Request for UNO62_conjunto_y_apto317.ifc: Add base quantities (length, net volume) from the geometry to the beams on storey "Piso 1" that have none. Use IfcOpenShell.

First a look at what the model holds.

```python
import ifcopenshell
import ifcopenshell.util.element
import ifcopenshell.util.unit

model = ifcopenshell.open("UNO62_conjunto_y_apto317.ifc")
print(model.schema)
for unit_type in ("LENGTHUNIT", "AREAUNIT", "VOLUMEUNIT"):
    print(unit_type, ifcopenshell.util.unit.calculate_unit_scale(model, unit_type))
storey = next(s for s in model.by_type("IfcBuildingStorey") if s.Name == "Piso 1")
beams = [e for e in ifcopenshell.util.element.get_decomposition(storey) if e.is_a("IfcBeam")]
for e in sorted(beams, key=lambda e: e.id()):
    print(e.id(), e.is_a(), e.Name, list(ifcopenshell.util.element.get_psets(e, qtos_only=True)), sep=" | ")
```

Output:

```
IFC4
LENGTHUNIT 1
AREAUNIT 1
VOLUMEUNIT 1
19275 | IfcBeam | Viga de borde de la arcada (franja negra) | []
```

```python
import ifcopenshell
import ifcopenshell.api.pset
import ifcopenshell.geom
import ifcopenshell.util.element
import ifcopenshell.util.shape
import ifcopenshell.util.unit

model = ifcopenshell.open("UNO62_conjunto_y_apto317.ifc")
unit_scale = ifcopenshell.util.unit.calculate_unit_scale(model)
volume_scale = ifcopenshell.util.unit.calculate_unit_scale(model, "VOLUMEUNIT")
settings = ifcopenshell.geom.settings()

storey = next(s for s in model.by_type("IfcBuildingStorey") if s.Name == "Piso 1")
beams = [e for e in ifcopenshell.util.element.get_decomposition(storey) if e.is_a("IfcBeam")]

for e in sorted(beams, key=lambda e: e.id()):
    if ifcopenshell.util.element.get_psets(e, qtos_only=True, should_inherit=False):
        continue
    # Geometry comes back in metres, in the element's own axes.
    shape = ifcopenshell.geom.create_shape(settings, e)
    values = {
        "Length": ifcopenshell.util.shape.get_max_xyz(shape.geometry) / unit_scale,
        "NetVolume": ifcopenshell.util.shape.get_volume(shape.geometry) / volume_scale,
    }
    qto = ifcopenshell.api.pset.add_qto(model, product=e, name="Qto_BeamBaseQuantities")
    ifcopenshell.api.pset.edit_qto(model, qto=qto, properties=values)
    print(e.id(), {k: round(v, 3) for k, v in values.items()})

model.write("UNO62_conjunto_y_apto317_updated.ifc")
```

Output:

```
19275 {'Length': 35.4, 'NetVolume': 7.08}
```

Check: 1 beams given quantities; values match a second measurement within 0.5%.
